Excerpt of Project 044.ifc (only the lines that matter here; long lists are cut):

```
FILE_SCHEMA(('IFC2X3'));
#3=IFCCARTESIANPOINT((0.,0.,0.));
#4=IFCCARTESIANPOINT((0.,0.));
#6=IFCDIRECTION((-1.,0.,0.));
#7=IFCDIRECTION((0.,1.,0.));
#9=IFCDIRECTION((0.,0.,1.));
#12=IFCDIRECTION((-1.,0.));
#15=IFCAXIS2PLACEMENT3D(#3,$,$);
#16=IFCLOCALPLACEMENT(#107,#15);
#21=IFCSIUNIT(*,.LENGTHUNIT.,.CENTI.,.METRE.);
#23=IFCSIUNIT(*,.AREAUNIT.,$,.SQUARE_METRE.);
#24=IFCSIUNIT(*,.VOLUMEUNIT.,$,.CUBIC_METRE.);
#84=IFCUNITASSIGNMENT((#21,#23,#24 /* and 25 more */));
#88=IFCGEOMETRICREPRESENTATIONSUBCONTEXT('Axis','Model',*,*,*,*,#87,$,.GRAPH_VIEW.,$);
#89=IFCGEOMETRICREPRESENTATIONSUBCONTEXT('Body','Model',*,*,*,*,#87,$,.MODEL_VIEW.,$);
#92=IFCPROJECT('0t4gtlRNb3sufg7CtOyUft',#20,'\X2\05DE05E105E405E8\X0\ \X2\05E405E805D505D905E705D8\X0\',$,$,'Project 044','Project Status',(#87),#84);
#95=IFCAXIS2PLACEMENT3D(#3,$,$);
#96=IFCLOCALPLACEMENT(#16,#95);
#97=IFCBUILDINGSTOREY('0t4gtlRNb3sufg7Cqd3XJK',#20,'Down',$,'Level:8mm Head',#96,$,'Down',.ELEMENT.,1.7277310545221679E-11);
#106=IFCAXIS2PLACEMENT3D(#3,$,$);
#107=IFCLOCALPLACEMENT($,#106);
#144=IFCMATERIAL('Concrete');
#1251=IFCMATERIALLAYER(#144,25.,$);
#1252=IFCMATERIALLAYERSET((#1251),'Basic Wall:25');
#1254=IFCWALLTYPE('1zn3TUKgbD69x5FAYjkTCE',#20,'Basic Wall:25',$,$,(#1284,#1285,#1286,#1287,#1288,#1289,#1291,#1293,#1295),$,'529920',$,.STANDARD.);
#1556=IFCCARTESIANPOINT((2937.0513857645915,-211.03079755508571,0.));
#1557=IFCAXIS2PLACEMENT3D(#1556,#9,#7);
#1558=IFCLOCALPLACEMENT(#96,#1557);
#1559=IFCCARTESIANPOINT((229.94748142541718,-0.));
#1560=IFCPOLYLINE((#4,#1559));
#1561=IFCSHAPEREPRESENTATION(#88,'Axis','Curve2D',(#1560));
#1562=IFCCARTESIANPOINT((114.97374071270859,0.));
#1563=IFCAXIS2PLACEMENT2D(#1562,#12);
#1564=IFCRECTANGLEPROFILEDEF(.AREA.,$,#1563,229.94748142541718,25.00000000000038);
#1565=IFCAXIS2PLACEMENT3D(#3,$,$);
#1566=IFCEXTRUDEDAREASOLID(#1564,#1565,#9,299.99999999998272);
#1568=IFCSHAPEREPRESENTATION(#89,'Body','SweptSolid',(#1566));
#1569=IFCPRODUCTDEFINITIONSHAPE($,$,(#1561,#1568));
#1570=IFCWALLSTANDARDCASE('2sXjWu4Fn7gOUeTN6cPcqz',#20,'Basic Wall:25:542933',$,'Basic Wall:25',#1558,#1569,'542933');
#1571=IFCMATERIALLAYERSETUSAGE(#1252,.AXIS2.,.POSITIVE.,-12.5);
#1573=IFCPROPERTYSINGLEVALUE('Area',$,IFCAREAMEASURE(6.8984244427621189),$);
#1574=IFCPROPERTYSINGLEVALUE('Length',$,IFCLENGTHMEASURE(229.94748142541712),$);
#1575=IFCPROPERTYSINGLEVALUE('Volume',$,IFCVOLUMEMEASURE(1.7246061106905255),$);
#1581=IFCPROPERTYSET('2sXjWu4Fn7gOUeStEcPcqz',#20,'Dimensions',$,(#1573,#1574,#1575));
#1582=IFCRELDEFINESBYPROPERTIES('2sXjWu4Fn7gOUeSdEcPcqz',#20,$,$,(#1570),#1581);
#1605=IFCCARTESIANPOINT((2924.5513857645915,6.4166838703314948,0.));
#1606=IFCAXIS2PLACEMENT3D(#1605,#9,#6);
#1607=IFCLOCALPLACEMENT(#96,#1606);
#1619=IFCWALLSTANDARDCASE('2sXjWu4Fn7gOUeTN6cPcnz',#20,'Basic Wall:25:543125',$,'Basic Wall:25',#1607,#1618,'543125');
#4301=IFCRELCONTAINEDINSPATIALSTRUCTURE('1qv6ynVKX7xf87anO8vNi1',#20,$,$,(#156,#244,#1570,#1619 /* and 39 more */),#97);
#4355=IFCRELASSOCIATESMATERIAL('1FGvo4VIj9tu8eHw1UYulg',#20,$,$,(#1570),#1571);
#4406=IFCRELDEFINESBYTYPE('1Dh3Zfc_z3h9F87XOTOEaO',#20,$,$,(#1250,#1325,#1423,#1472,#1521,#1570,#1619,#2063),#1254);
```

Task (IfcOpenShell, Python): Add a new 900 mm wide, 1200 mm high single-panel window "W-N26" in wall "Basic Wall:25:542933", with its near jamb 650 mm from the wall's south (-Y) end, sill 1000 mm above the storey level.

```python
import numpy as np
import ifcopenshell
import ifcopenshell.api.feature
import ifcopenshell.api.geometry
import ifcopenshell.api.pset
import ifcopenshell.api.root
import ifcopenshell.api.spatial
import ifcopenshell.api.type
import ifcopenshell.geom
import ifcopenshell.util.element
import ifcopenshell.util.placement
import ifcopenshell.util.representation
import ifcopenshell.util.shape
import ifcopenshell.util.unit

model = ifcopenshell.open("Project 044.ifc")
unit_scale = ifcopenshell.util.unit.calculate_unit_scale(model)
area_scale = ifcopenshell.util.unit.calculate_unit_scale(model, "AREAUNIT")
volume_scale = ifcopenshell.util.unit.calculate_unit_scale(model, "VOLUMEUNIT")
settings = ifcopenshell.geom.settings()


def volume(element):
    """Net volume in cubic metres, openings subtracted."""
    shape = ifcopenshell.geom.create_shape(settings, element)
    return ifcopenshell.util.shape.get_volume(shape.geometry)


wall = model.by_id(1570)
storey = ifcopenshell.util.element.get_container(wall, ifc_class="IfcBuildingStorey")
context = ifcopenshell.util.representation.get_context(model, "Model", "Body", "MODEL_VIEW")
before = volume(wall)

width, height, from_end, sill = 0.9, 1.2, 0.65, 1  # metres

# The wall runs along its own X axis, and the end named is its -X end.
wall_shape = ifcopenshell.geom.create_shape(settings, wall)
x, y, z = ifcopenshell.util.shape.get_vertices(wall_shape.geometry).T
start = x.min() + from_end
face, thickness = float(y.min()), float(y.max() - y.min())
wall_matrix = ifcopenshell.util.placement.get_local_placement(wall.ObjectPlacement)
level = ifcopenshell.util.placement.get_local_placement(storey.ObjectPlacement)[2, 3]


def in_wall(x, y):
    """Placement at x, y metres in the wall's axes, at sill height."""
    matrix = wall_matrix.copy()
    matrix[:, 3] = wall_matrix @ np.array([x / unit_scale, y / unit_scale, 0.0, 1.0])
    matrix[2, 3] = level + sill / unit_scale
    return matrix


# Opening: a box that overshoots both wall faces by 50 mm.
opening = ifcopenshell.api.root.create_entity(model, ifc_class="IfcOpeningElement")
box = ifcopenshell.api.geometry.add_wall_representation(
    model, context=context, length=width, height=height, thickness=thickness + 0.1
)
ifcopenshell.api.geometry.assign_representation(model, product=opening, representation=box)
ifcopenshell.api.geometry.edit_object_placement(model, product=opening, matrix=in_wall(start, face - 0.05), is_si=False)
ifcopenshell.api.feature.add_feature(model, feature=opening, element=wall)

window = ifcopenshell.api.root.create_entity(model, ifc_class="IfcWindow", name="W-N26")
window.OverallWidth, window.OverallHeight = width / unit_scale, height / unit_scale
body = ifcopenshell.api.geometry.add_window_representation(
    model,
    context=context,
    overall_width=window.OverallWidth,
    overall_height=window.OverallHeight,
    partition_type="SINGLE_PANEL",
)
ifcopenshell.api.geometry.assign_representation(model, product=window, representation=body)
ifcopenshell.api.spatial.assign_container(model, products=[window], relating_structure=storey)
fills = ifcopenshell.api.feature.add_filling(model, opening=opening, element=window)
fills.OwnerHistory = window.OwnerHistory  # required in IFC2X3

# IFC2X3 keeps the operation on the window style.
style = ifcopenshell.api.root.create_entity(model, ifc_class="IfcWindowStyle", name="W-N26")
style.OperationType, style.ConstructionType = "SINGLE_PANEL", "NOTDEFINED"
style.ParameterTakesPrecedence = style.Sizeable = False
ifcopenshell.api.type.assign_type(model, related_objects=[window], relating_type=style)

# Centre the window in the wall's thickness.
ifcopenshell.api.geometry.edit_object_placement(model, product=window, matrix=in_wall(start, face), is_si=False)
window_shape = ifcopenshell.geom.create_shape(settings, window)
depth = ifcopenshell.util.shape.get_vertices(window_shape.geometry)[:, 1]
offset = face + thickness / 2 - (depth.min() + depth.max()) / 2
ifcopenshell.api.geometry.edit_object_placement(model, product=window, matrix=in_wall(start, offset), is_si=False)

after = volume(wall)

# Update the wall's stored quantities.
pset = model.by_id(ifcopenshell.util.element.get_pset(wall, "Dimensions", should_inherit=False)["id"])
ifcopenshell.api.pset.edit_pset(model, pset=pset, properties={
    "Area": model.create_entity("IfcAreaMeasure", after / thickness / area_scale),
    "Volume": model.create_entity("IfcVolumeMeasure", after / volume_scale),
})

print(f"wall volume {before:.3f} -> {after:.3f} m3")

model.write("Project 044_updated.ifc")
```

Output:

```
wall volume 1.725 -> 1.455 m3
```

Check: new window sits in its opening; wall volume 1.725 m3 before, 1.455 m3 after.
